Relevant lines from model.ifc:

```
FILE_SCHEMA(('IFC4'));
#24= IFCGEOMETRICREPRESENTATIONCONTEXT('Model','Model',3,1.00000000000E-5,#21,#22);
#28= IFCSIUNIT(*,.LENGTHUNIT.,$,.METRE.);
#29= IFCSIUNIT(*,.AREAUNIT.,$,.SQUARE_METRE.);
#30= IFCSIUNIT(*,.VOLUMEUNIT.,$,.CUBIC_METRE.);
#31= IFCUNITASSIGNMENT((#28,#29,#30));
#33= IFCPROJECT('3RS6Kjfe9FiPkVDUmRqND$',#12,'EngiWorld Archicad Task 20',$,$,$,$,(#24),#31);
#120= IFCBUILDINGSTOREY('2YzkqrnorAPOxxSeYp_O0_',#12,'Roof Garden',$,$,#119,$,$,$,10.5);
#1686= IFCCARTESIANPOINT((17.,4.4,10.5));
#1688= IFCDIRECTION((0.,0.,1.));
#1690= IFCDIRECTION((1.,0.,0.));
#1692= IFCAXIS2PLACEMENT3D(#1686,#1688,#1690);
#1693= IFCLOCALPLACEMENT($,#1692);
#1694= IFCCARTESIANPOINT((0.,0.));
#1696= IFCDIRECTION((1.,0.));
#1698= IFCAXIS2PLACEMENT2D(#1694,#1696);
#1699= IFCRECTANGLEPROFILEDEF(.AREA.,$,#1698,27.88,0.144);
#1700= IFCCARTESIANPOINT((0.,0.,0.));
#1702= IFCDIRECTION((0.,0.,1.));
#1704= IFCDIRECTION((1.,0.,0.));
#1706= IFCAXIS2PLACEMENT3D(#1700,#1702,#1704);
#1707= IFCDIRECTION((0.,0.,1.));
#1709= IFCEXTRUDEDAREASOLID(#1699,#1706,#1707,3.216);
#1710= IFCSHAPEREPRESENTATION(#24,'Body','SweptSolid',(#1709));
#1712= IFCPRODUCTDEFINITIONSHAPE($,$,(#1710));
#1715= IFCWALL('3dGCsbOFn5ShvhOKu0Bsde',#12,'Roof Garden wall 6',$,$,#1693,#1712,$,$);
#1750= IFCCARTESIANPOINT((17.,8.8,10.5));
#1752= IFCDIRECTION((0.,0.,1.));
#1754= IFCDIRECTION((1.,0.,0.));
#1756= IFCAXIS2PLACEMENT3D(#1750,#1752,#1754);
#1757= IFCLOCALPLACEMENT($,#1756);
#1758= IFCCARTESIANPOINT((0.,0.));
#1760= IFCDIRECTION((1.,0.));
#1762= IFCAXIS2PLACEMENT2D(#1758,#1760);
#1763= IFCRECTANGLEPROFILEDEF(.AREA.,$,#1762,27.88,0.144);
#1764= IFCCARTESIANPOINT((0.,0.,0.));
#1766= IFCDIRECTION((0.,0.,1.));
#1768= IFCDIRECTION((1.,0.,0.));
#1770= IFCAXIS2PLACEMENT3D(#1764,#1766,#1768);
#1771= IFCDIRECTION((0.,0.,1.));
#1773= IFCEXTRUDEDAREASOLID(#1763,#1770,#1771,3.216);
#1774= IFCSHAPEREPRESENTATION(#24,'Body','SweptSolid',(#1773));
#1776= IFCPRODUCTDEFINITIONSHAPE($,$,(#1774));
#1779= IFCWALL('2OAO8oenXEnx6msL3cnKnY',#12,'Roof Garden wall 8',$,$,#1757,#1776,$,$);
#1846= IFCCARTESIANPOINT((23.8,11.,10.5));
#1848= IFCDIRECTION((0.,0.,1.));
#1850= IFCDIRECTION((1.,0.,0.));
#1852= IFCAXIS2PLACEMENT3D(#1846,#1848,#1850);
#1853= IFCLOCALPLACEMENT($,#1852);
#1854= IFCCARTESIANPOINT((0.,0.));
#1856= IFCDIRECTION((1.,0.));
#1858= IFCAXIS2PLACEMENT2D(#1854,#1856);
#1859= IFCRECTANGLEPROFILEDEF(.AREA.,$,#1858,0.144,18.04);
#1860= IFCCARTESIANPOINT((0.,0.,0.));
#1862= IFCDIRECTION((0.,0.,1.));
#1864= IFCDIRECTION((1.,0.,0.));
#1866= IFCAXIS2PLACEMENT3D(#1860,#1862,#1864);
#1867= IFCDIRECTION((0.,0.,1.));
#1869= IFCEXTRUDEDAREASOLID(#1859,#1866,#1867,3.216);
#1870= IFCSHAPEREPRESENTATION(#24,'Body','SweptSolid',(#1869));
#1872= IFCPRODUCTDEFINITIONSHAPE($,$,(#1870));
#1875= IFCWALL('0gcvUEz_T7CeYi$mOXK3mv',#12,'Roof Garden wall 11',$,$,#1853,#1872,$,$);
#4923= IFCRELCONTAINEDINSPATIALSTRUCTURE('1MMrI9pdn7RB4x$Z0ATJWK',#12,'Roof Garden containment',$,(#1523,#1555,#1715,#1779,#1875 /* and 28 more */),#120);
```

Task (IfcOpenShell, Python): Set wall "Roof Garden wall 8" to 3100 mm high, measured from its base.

```python
import ifcopenshell
import ifcopenshell.geom
import ifcopenshell.util.shape
import ifcopenshell.util.unit

model = ifcopenshell.open("model.ifc")
unit_scale = ifcopenshell.util.unit.calculate_unit_scale(model)
settings = ifcopenshell.geom.settings()


def volume(element):
    """Net volume in cubic metres, openings subtracted."""
    shape = ifcopenshell.geom.create_shape(settings, element)
    return ifcopenshell.util.shape.get_volume(shape.geometry)


wall = model.by_id(1779)
before = volume(wall)

body = next(r for r in wall.Representation.Representations if r.RepresentationIdentifier == "Body")
solid = body.Items[0]
old_height = solid.Depth
solid.Depth = 3.1 / unit_scale
after = volume(wall)

print(f"height {old_height:g} -> {solid.Depth:g}, volume {before:.3f} -> {after:.3f} m3")

model.write("model_edited.ifc")
```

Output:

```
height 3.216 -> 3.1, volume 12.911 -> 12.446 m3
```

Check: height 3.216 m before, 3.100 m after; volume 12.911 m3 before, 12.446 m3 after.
